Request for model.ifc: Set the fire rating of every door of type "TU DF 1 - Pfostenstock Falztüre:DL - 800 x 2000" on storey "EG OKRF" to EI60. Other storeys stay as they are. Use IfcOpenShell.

First a look at what the model holds.

```python
import ifcopenshell
import ifcopenshell.util.element

model = ifcopenshell.open("model.ifc")
print(model.schema)
storey = next(s for s in model.by_type("IfcBuildingStorey") if s.Name == "EG OKRF")
doors = [e for e in ifcopenshell.util.element.get_decomposition(storey) if e.is_a("IfcDoor")]
seen = {}
for e in doors:
    element_type = ifcopenshell.util.element.get_type(e)
    key = (element_type.Name if element_type != e and element_type else None, ifcopenshell.util.element.get_pset(e, "Pset_DoorCommon", "FireRating"))
    seen[key] = seen.get(key, 0) + 1
for (name, value), count in sorted(seen.items(), key=str):
    print(count, "x", name, "|", value)
```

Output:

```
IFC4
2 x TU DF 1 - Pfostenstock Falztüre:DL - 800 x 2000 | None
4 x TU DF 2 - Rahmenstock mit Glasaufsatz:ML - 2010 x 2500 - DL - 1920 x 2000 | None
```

```python
import ifcopenshell
import ifcopenshell.api.pset
import ifcopenshell.util.element

model = ifcopenshell.open("model.ifc")

storey = next(s for s in model.by_type("IfcBuildingStorey") if s.Name == "EG OKRF")
doors = [e for e in ifcopenshell.util.element.get_decomposition(storey) if e.is_a("IfcDoor")]

count = 0
for e in doors:
    element_type = ifcopenshell.util.element.get_type(e)
    if element_type in (None, e) or element_type.Name != "TU DF 1 - Pfostenstock Falztüre:DL - 800 x 2000":
        continue
    # add_pset returns the element's existing set when there is one.
    pset = ifcopenshell.api.pset.add_pset(model, product=e, name="Pset_DoorCommon")
    ifcopenshell.api.pset.edit_pset(model, pset=pset, properties={"FireRating": "EI60"})
    count += 1

print(count, "doors updated")

model.write("model_v2.ifc")
```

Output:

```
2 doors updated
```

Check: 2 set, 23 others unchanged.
